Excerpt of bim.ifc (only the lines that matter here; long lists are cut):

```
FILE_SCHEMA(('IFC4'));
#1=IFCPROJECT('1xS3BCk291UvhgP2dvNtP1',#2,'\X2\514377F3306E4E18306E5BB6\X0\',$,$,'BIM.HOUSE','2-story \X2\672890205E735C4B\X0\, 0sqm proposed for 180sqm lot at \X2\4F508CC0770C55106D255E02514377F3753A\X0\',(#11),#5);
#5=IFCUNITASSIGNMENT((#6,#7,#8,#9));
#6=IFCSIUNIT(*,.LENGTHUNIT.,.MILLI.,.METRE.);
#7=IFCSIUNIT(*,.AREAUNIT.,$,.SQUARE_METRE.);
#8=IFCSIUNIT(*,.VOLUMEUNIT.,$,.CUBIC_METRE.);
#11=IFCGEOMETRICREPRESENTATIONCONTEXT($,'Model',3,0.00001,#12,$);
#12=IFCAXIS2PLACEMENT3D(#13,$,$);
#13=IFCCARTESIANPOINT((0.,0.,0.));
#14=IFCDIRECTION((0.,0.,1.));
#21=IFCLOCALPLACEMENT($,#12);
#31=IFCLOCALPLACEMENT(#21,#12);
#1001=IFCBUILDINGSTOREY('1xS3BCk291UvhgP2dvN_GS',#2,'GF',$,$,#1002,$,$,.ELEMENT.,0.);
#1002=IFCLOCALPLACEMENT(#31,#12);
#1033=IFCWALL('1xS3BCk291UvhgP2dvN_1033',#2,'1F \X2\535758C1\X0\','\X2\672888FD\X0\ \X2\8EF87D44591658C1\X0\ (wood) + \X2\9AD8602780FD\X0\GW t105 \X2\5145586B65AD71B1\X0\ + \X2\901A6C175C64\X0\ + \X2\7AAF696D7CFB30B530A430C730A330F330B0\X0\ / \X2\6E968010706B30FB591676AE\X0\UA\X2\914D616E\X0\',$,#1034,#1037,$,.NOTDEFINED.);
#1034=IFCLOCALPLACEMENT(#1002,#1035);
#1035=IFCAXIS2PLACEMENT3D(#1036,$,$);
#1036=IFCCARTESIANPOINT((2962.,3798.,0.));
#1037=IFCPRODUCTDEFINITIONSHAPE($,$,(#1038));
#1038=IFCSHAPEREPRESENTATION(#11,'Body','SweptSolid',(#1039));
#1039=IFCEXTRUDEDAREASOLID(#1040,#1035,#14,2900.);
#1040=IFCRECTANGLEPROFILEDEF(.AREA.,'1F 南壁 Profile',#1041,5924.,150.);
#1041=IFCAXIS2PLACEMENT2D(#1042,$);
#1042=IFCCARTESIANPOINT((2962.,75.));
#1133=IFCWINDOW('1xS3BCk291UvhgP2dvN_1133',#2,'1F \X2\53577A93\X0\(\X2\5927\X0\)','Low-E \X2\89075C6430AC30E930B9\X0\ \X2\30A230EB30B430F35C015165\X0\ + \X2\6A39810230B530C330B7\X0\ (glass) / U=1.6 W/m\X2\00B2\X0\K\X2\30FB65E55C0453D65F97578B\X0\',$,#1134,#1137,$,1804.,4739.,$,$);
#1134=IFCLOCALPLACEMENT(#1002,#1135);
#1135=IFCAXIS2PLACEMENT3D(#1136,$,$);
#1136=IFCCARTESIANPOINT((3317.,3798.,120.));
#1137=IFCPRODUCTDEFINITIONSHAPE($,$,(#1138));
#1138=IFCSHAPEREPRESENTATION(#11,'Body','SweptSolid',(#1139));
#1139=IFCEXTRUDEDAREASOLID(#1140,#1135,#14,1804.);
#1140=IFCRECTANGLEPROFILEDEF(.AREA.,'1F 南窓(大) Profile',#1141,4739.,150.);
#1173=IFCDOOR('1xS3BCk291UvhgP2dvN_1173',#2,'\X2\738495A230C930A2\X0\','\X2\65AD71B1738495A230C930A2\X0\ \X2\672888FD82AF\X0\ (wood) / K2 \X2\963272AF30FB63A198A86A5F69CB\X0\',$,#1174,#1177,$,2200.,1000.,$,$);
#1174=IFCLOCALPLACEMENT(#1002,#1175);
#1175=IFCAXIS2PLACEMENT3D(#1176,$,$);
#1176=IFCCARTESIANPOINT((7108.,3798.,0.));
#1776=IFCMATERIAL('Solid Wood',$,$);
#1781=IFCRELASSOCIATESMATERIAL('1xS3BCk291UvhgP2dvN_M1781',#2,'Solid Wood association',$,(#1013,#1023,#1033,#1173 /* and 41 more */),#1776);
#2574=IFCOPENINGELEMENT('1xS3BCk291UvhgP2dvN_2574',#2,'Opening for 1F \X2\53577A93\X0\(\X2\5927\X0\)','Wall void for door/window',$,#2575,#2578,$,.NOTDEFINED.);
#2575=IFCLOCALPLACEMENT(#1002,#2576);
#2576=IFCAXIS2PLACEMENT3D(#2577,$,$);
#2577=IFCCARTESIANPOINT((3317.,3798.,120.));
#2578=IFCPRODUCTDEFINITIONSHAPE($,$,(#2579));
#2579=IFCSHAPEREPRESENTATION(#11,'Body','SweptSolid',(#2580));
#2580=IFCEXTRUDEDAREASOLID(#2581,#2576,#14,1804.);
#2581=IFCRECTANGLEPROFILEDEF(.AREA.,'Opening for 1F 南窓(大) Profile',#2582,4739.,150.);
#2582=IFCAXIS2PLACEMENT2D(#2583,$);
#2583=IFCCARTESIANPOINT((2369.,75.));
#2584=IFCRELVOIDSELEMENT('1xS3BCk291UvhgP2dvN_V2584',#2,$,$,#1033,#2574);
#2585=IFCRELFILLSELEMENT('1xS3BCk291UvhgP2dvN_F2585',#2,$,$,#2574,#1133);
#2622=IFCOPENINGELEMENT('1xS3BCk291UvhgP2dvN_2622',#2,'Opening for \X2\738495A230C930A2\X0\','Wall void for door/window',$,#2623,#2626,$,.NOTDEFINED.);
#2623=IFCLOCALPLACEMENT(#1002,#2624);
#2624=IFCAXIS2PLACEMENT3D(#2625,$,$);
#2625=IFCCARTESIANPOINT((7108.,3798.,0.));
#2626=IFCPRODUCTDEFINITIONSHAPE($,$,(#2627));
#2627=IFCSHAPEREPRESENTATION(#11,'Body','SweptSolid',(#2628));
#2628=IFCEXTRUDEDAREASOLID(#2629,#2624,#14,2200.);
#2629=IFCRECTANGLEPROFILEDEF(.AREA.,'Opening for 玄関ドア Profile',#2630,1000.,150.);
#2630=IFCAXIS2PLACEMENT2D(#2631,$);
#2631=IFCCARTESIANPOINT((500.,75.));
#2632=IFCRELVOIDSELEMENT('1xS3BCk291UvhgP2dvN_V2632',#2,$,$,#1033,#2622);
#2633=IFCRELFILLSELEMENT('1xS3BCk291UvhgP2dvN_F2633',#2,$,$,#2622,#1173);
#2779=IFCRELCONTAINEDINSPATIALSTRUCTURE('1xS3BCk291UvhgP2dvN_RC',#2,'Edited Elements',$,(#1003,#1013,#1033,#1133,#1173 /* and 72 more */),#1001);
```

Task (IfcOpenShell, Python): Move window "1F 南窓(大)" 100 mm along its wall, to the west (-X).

```python
import ifcopenshell
import ifcopenshell.api.geometry
import ifcopenshell.util.placement

model = ifcopenshell.open("bim.ifc")

window = model.by_guid("1xS3BCk291UvhgP2dvN_1133")
opening = window.FillsVoids[0].RelatingOpeningElement
wall = opening.VoidsElements[0].RelatingBuildingElement

wall_matrix = ifcopenshell.util.placement.get_local_placement(wall.ObjectPlacement)
shift = wall_matrix[:3, 0] * -100.0
before = ifcopenshell.util.placement.get_local_placement(window.ObjectPlacement)[:3, 3].copy()

# The window is not placed relative to its opening, so move both.
for product in (opening, window):
    matrix = ifcopenshell.util.placement.get_local_placement(product.ObjectPlacement)
    matrix[:3, 3] += shift
    ifcopenshell.api.geometry.edit_object_placement(model, product=product, matrix=matrix, is_si=False)

after = ifcopenshell.util.placement.get_local_placement(window.ObjectPlacement)[:3, 3]
print("window moved by", (after - before).round(3) + 0.0)

model.write("bim_updated.ifc")
```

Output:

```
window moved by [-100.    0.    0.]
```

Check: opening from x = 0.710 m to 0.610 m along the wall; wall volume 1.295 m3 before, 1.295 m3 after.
